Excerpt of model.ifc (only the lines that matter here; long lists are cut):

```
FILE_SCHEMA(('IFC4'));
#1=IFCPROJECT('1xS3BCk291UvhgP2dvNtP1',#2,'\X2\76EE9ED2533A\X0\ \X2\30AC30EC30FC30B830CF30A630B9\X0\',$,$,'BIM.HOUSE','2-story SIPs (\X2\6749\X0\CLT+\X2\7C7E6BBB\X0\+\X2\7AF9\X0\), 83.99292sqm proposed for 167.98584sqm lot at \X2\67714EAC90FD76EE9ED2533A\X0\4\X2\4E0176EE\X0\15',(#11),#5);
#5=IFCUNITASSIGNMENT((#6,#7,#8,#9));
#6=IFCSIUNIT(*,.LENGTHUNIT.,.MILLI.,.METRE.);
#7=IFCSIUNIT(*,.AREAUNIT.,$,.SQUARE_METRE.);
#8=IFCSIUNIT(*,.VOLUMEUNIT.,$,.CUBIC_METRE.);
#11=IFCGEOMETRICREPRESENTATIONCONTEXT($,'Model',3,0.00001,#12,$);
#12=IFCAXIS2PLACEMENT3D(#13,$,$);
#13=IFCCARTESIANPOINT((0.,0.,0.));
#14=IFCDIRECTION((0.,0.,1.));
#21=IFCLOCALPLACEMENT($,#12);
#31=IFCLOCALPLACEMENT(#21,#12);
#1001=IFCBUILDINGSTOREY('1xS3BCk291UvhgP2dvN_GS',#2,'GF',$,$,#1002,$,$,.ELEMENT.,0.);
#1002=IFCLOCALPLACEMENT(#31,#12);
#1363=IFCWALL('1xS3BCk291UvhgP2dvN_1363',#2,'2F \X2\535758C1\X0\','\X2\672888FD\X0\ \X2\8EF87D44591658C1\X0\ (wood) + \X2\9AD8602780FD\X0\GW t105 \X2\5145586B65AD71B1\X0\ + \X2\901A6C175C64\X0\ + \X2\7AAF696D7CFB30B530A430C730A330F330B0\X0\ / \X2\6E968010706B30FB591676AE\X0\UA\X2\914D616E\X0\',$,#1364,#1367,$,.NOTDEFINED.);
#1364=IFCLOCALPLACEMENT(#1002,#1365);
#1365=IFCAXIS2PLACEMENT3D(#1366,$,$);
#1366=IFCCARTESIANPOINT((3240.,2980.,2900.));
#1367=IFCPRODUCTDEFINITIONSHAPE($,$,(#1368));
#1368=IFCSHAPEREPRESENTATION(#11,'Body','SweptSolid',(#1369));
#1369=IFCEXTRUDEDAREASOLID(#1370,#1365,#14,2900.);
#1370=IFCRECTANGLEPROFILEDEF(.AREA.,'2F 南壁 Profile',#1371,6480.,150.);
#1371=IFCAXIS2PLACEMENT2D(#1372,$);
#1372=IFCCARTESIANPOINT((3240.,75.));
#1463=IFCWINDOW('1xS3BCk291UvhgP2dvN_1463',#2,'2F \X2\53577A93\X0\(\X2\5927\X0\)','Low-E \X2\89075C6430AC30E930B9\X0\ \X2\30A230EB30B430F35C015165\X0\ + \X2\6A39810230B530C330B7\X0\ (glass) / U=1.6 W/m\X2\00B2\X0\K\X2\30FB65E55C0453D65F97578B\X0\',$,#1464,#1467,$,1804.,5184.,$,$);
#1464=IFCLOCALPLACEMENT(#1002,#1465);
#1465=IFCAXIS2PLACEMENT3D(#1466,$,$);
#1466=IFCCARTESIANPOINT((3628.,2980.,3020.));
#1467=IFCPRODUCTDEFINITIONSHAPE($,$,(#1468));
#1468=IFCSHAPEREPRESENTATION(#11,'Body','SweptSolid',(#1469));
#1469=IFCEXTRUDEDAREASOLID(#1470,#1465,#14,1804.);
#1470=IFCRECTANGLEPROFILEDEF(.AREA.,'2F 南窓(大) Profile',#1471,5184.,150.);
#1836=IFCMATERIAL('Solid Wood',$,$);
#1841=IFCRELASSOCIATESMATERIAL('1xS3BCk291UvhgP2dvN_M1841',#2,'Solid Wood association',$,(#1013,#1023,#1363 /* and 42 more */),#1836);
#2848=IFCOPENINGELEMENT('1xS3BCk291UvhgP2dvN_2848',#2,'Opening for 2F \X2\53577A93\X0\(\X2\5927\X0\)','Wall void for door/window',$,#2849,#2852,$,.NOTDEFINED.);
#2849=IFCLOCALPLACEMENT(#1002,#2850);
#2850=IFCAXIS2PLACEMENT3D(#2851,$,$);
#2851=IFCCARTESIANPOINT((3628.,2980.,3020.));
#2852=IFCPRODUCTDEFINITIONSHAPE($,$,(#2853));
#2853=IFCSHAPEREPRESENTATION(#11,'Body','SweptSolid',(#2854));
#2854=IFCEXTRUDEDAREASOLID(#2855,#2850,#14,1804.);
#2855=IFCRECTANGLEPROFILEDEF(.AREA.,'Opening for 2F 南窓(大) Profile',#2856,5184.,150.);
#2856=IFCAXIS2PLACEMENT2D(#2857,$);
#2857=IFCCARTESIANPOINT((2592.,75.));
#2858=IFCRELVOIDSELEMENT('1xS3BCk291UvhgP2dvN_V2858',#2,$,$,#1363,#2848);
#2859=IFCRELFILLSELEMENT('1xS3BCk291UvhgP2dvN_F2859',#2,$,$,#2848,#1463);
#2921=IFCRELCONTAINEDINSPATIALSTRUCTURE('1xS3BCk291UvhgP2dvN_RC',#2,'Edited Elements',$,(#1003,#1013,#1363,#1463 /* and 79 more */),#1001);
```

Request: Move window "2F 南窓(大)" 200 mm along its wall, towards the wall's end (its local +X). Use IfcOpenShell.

```python
import ifcopenshell
import ifcopenshell.api.geometry
import ifcopenshell.util.placement
import ifcopenshell.util.unit

model = ifcopenshell.open("model.ifc")
unit_scale = ifcopenshell.util.unit.calculate_unit_scale(model)

window = model.by_id(1463)
opening = window.FillsVoids[0].RelatingOpeningElement
wall = opening.VoidsElements[0].RelatingBuildingElement

wall_matrix = ifcopenshell.util.placement.get_local_placement(wall.ObjectPlacement)
shift = wall_matrix[:3, 0] * 0.2 / unit_scale
before = ifcopenshell.util.placement.get_local_placement(window.ObjectPlacement)[:3, 3].copy()

# The window is not placed relative to its opening, so move both.
for product in (opening, window):
    matrix = ifcopenshell.util.placement.get_local_placement(product.ObjectPlacement)
    matrix[:3, 3] += shift
    ifcopenshell.api.geometry.edit_object_placement(model, product=product, matrix=matrix, is_si=False)

after = ifcopenshell.util.placement.get_local_placement(window.ObjectPlacement)[:3, 3]
print("window moved by", (after - before).round(3) + 0.0)

model.write("model_updated.ifc")
```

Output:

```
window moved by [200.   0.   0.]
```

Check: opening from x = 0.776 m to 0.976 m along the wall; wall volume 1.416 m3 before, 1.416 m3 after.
